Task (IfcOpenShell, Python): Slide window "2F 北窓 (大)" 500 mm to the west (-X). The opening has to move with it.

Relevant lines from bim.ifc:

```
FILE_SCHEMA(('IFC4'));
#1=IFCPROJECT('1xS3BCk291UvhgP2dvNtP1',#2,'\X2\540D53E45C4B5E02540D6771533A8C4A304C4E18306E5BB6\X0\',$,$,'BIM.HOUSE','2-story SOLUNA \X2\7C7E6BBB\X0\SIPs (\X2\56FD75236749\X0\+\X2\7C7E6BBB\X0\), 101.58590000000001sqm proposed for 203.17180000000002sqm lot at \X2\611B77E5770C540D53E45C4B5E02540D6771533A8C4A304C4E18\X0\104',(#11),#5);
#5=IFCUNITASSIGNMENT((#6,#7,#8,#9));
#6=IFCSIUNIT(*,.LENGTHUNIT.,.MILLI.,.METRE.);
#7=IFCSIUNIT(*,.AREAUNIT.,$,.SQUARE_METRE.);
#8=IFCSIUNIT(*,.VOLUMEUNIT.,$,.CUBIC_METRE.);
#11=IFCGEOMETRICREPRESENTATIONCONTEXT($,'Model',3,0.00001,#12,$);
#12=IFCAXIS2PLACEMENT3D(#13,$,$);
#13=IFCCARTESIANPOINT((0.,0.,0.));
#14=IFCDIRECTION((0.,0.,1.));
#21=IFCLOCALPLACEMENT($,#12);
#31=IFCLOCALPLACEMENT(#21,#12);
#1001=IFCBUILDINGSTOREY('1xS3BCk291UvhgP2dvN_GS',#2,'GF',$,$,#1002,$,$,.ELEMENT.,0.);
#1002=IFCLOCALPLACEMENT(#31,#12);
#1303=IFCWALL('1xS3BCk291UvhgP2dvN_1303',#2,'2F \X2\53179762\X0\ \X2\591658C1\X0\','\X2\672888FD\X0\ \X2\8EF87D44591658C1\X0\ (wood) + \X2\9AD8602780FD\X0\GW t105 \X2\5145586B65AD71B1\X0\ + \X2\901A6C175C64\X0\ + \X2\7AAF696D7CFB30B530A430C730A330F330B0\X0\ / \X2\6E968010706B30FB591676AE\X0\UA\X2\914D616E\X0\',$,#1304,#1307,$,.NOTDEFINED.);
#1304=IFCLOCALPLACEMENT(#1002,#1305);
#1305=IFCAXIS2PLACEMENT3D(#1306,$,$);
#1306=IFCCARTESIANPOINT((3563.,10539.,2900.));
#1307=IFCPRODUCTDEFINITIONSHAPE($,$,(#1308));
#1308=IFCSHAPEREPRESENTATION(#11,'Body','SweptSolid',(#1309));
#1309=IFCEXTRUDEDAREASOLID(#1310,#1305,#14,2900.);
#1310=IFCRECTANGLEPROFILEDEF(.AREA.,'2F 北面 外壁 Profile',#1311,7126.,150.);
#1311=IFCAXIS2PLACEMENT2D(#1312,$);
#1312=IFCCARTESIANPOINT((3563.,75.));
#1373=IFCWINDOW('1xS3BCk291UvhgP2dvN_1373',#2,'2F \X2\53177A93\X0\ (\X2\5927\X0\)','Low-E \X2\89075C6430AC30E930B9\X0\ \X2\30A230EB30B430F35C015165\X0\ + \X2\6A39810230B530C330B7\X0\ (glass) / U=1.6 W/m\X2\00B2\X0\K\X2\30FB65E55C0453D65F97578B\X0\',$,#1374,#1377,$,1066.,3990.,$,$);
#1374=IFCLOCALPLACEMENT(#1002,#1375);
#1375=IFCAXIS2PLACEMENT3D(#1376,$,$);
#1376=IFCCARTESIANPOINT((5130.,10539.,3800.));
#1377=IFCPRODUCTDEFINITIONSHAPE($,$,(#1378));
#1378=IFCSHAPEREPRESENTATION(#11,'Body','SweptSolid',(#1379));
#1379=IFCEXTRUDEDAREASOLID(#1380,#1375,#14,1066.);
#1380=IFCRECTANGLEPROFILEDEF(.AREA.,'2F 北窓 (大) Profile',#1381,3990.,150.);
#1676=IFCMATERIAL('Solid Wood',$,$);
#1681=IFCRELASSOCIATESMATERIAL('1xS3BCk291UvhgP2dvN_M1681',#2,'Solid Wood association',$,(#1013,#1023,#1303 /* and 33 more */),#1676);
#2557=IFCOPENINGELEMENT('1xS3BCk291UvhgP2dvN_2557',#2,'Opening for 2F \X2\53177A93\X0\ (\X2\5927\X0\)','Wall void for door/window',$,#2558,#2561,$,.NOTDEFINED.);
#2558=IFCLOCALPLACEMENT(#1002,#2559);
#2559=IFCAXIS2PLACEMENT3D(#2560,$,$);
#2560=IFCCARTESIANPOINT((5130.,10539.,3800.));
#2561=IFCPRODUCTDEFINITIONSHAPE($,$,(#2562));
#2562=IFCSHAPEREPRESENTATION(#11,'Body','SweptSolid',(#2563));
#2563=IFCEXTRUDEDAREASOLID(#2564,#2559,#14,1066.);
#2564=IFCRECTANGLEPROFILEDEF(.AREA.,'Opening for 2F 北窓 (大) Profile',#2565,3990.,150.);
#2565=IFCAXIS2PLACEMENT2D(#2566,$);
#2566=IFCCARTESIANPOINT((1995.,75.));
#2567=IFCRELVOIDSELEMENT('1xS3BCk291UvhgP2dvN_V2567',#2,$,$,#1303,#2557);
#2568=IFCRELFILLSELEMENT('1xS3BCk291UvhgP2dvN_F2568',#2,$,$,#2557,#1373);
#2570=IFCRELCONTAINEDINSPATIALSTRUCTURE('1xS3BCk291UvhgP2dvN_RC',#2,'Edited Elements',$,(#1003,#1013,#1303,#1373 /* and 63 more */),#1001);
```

```python
import ifcopenshell
import ifcopenshell.api.geometry
import ifcopenshell.util.placement
import ifcopenshell.util.unit

model = ifcopenshell.open("bim.ifc")
unit_scale = ifcopenshell.util.unit.calculate_unit_scale(model)

window = model.by_id(1373)
opening = window.FillsVoids[0].RelatingOpeningElement
wall = opening.VoidsElements[0].RelatingBuildingElement

wall_matrix = ifcopenshell.util.placement.get_local_placement(wall.ObjectPlacement)
shift = wall_matrix[:3, 0] * -0.5 / unit_scale
before = ifcopenshell.util.placement.get_local_placement(window.ObjectPlacement)[:3, 3].copy()

# The window is not placed relative to its opening, so move both.
for product in (opening, window):
    matrix = ifcopenshell.util.placement.get_local_placement(product.ObjectPlacement)
    matrix[:3, 3] += shift
    ifcopenshell.api.geometry.edit_object_placement(model, product=product, matrix=matrix, is_si=False)

after = ifcopenshell.util.placement.get_local_placement(window.ObjectPlacement)[:3, 3]
print("window moved by", (after - before).round(3) + 0.0)

model.write("bim_edited.ifc")
```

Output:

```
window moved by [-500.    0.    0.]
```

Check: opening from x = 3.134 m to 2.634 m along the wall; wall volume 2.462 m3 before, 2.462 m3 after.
